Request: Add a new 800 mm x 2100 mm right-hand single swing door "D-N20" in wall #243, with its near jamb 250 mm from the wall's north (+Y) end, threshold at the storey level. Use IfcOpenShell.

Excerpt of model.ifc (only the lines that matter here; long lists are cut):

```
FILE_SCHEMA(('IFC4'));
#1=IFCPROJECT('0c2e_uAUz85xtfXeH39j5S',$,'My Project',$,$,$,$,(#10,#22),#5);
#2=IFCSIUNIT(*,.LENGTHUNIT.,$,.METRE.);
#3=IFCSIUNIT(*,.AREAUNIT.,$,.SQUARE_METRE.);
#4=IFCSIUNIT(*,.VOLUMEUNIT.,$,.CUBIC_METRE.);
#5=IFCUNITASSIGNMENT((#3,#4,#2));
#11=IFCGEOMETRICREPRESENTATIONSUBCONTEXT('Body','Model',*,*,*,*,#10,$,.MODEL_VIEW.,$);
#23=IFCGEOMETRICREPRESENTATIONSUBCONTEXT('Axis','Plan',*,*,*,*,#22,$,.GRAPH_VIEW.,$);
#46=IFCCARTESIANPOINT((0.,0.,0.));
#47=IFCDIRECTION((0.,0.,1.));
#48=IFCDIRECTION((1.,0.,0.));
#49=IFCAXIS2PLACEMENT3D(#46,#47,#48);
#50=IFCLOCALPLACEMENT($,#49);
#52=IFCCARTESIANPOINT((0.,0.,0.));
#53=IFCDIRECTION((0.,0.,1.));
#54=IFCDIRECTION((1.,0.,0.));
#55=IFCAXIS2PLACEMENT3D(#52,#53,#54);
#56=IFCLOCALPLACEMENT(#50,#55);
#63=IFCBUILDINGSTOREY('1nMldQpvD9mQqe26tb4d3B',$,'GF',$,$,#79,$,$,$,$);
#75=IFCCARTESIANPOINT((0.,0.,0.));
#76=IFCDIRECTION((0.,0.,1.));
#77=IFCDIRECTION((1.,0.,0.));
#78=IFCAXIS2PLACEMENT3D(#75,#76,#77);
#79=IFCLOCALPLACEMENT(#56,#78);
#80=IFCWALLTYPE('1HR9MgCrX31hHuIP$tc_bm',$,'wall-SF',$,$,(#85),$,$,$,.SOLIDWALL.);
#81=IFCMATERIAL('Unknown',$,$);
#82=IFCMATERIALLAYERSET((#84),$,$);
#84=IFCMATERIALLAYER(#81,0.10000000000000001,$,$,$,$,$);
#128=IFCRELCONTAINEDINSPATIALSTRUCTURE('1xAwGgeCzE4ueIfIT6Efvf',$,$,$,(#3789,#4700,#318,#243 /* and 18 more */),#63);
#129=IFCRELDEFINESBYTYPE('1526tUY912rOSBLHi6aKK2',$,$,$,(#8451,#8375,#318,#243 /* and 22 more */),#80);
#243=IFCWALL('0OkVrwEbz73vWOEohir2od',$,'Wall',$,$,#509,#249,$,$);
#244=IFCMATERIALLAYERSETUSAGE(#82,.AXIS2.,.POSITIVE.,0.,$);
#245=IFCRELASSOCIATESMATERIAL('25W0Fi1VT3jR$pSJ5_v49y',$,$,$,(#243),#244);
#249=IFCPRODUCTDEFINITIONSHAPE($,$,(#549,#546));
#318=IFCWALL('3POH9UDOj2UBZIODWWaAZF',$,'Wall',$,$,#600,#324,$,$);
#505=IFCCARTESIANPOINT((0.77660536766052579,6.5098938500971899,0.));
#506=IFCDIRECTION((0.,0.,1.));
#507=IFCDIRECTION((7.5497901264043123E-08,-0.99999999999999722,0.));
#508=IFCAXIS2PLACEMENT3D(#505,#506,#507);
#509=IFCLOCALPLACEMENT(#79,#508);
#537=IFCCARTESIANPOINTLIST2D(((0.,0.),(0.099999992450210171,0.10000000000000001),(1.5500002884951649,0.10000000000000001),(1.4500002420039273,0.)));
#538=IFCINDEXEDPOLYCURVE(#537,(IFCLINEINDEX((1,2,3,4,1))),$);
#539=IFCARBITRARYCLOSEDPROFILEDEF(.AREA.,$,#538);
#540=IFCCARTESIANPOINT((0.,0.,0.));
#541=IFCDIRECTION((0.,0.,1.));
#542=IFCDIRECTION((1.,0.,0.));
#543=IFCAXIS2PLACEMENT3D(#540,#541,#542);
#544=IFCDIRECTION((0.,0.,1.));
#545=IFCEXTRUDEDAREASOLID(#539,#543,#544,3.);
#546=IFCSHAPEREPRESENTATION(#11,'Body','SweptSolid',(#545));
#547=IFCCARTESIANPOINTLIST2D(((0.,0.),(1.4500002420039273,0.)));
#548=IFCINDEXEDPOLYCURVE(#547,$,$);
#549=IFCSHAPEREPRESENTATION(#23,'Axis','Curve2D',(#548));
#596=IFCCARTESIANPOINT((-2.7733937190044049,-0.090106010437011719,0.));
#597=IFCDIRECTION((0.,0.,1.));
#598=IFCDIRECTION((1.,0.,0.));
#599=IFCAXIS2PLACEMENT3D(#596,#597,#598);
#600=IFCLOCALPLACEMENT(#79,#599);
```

```python
import numpy as np
import ifcopenshell
import ifcopenshell.api.feature
import ifcopenshell.api.geometry
import ifcopenshell.api.root
import ifcopenshell.api.spatial
import ifcopenshell.geom
import ifcopenshell.util.element
import ifcopenshell.util.placement
import ifcopenshell.util.representation
import ifcopenshell.util.shape
import ifcopenshell.util.unit

model = ifcopenshell.open("model.ifc")
unit_scale = ifcopenshell.util.unit.calculate_unit_scale(model)
settings = ifcopenshell.geom.settings()


def volume(element):
    """Net volume in cubic metres, openings subtracted."""
    shape = ifcopenshell.geom.create_shape(settings, element)
    return ifcopenshell.util.shape.get_volume(shape.geometry)


wall = model.by_guid("0OkVrwEbz73vWOEohir2od")
storey = ifcopenshell.util.element.get_container(wall, ifc_class="IfcBuildingStorey")
context = ifcopenshell.util.representation.get_context(model, "Model", "Body", "MODEL_VIEW")
before = volume(wall)

width, height, from_end, sill = 0.8, 2.1, 0.25, 0.0  # metres

# The wall runs along its own X axis, and the end named is its -X end.
wall_shape = ifcopenshell.geom.create_shape(settings, wall)
x, y, z = ifcopenshell.util.shape.get_vertices(wall_shape.geometry).T
start = x.min() + from_end
face, thickness = float(y.min()), float(y.max() - y.min())
wall_matrix = ifcopenshell.util.placement.get_local_placement(wall.ObjectPlacement)
level = ifcopenshell.util.placement.get_local_placement(storey.ObjectPlacement)[2, 3]


def in_wall(x, y):
    """Placement at x, y metres in the wall's axes, at sill height."""
    matrix = wall_matrix.copy()
    matrix[:, 3] = wall_matrix @ np.array([x / unit_scale, y / unit_scale, 0.0, 1.0])
    matrix[2, 3] = level + sill / unit_scale
    return matrix


# Opening: a box that overshoots both wall faces by 50 mm.
opening = ifcopenshell.api.root.create_entity(model, ifc_class="IfcOpeningElement", predefined_type="OPENING")
box = ifcopenshell.api.geometry.add_wall_representation(
    model, context=context, length=width, height=height, thickness=thickness + 0.1
)
ifcopenshell.api.geometry.assign_representation(model, product=opening, representation=box)
ifcopenshell.api.geometry.edit_object_placement(model, product=opening, matrix=in_wall(start, face - 0.05), is_si=False)
ifcopenshell.api.feature.add_feature(model, feature=opening, element=wall)

door = ifcopenshell.api.root.create_entity(model, ifc_class="IfcDoor", name="D-N20", predefined_type="DOOR")
door.OverallWidth, door.OverallHeight = width / unit_scale, height / unit_scale
door.OperationType = "SINGLE_SWING_RIGHT"
body = ifcopenshell.api.geometry.add_door_representation(
    model,
    context=context,
    overall_width=door.OverallWidth,
    overall_height=door.OverallHeight,
    operation_type="SINGLE_SWING_RIGHT",
    lining_properties={"LiningDepth": thickness / unit_scale, "ThresholdDepth": thickness / unit_scale},
)
ifcopenshell.api.geometry.assign_representation(model, product=door, representation=body)
ifcopenshell.api.spatial.assign_container(model, products=[door], relating_structure=storey)
ifcopenshell.api.feature.add_filling(model, opening=opening, element=door)

# The lining spans the wall, so the door starts at the wall face.
ifcopenshell.api.geometry.edit_object_placement(model, product=door, matrix=in_wall(start, face), is_si=False)

after = volume(wall)

print(f"wall volume {before:.3f} -> {after:.3f} m3")

model.write("model-out.ifc")
```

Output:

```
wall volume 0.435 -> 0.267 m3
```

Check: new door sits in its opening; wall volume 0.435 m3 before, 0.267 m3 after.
